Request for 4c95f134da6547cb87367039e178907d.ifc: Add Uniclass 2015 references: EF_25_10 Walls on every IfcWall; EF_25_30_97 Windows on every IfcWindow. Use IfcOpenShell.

First a look at what the model holds.

```python
import ifcopenshell

model = ifcopenshell.open("4c95f134da6547cb87367039e178907d.ifc")
print(model.schema)
print("classifications:", [c.Name for c in model.by_type("IfcClassification")])
for ifc_class in ("IfcDoor", "IfcRoof", "IfcStair", "IfcWall", "IfcWindow"):
    print(ifc_class, len(model.by_type(ifc_class)))
```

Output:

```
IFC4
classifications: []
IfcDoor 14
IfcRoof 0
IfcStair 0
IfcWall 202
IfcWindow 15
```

```python
import ifcopenshell
import ifcopenshell.api.classification

model = ifcopenshell.open("4c95f134da6547cb87367039e178907d.ifc")

system = ifcopenshell.api.classification.add_classification(model, classification="Uniclass 2015")

codes = {
    "IfcWall": ("EF_25_10", "Walls"),
    "IfcWindow": ("EF_25_30_97", "Windows"),
}
for ifc_class, (code, name) in codes.items():
    products = model.by_type(ifc_class)
    ifcopenshell.api.classification.add_reference(
        model, products=products, classification=system, identification=code, name=name
    )
    print(code, len(products))

model.write("4c95f134da6547cb87367039e178907d_edited.ifc")
```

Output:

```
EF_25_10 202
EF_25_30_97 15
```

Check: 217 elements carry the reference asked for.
